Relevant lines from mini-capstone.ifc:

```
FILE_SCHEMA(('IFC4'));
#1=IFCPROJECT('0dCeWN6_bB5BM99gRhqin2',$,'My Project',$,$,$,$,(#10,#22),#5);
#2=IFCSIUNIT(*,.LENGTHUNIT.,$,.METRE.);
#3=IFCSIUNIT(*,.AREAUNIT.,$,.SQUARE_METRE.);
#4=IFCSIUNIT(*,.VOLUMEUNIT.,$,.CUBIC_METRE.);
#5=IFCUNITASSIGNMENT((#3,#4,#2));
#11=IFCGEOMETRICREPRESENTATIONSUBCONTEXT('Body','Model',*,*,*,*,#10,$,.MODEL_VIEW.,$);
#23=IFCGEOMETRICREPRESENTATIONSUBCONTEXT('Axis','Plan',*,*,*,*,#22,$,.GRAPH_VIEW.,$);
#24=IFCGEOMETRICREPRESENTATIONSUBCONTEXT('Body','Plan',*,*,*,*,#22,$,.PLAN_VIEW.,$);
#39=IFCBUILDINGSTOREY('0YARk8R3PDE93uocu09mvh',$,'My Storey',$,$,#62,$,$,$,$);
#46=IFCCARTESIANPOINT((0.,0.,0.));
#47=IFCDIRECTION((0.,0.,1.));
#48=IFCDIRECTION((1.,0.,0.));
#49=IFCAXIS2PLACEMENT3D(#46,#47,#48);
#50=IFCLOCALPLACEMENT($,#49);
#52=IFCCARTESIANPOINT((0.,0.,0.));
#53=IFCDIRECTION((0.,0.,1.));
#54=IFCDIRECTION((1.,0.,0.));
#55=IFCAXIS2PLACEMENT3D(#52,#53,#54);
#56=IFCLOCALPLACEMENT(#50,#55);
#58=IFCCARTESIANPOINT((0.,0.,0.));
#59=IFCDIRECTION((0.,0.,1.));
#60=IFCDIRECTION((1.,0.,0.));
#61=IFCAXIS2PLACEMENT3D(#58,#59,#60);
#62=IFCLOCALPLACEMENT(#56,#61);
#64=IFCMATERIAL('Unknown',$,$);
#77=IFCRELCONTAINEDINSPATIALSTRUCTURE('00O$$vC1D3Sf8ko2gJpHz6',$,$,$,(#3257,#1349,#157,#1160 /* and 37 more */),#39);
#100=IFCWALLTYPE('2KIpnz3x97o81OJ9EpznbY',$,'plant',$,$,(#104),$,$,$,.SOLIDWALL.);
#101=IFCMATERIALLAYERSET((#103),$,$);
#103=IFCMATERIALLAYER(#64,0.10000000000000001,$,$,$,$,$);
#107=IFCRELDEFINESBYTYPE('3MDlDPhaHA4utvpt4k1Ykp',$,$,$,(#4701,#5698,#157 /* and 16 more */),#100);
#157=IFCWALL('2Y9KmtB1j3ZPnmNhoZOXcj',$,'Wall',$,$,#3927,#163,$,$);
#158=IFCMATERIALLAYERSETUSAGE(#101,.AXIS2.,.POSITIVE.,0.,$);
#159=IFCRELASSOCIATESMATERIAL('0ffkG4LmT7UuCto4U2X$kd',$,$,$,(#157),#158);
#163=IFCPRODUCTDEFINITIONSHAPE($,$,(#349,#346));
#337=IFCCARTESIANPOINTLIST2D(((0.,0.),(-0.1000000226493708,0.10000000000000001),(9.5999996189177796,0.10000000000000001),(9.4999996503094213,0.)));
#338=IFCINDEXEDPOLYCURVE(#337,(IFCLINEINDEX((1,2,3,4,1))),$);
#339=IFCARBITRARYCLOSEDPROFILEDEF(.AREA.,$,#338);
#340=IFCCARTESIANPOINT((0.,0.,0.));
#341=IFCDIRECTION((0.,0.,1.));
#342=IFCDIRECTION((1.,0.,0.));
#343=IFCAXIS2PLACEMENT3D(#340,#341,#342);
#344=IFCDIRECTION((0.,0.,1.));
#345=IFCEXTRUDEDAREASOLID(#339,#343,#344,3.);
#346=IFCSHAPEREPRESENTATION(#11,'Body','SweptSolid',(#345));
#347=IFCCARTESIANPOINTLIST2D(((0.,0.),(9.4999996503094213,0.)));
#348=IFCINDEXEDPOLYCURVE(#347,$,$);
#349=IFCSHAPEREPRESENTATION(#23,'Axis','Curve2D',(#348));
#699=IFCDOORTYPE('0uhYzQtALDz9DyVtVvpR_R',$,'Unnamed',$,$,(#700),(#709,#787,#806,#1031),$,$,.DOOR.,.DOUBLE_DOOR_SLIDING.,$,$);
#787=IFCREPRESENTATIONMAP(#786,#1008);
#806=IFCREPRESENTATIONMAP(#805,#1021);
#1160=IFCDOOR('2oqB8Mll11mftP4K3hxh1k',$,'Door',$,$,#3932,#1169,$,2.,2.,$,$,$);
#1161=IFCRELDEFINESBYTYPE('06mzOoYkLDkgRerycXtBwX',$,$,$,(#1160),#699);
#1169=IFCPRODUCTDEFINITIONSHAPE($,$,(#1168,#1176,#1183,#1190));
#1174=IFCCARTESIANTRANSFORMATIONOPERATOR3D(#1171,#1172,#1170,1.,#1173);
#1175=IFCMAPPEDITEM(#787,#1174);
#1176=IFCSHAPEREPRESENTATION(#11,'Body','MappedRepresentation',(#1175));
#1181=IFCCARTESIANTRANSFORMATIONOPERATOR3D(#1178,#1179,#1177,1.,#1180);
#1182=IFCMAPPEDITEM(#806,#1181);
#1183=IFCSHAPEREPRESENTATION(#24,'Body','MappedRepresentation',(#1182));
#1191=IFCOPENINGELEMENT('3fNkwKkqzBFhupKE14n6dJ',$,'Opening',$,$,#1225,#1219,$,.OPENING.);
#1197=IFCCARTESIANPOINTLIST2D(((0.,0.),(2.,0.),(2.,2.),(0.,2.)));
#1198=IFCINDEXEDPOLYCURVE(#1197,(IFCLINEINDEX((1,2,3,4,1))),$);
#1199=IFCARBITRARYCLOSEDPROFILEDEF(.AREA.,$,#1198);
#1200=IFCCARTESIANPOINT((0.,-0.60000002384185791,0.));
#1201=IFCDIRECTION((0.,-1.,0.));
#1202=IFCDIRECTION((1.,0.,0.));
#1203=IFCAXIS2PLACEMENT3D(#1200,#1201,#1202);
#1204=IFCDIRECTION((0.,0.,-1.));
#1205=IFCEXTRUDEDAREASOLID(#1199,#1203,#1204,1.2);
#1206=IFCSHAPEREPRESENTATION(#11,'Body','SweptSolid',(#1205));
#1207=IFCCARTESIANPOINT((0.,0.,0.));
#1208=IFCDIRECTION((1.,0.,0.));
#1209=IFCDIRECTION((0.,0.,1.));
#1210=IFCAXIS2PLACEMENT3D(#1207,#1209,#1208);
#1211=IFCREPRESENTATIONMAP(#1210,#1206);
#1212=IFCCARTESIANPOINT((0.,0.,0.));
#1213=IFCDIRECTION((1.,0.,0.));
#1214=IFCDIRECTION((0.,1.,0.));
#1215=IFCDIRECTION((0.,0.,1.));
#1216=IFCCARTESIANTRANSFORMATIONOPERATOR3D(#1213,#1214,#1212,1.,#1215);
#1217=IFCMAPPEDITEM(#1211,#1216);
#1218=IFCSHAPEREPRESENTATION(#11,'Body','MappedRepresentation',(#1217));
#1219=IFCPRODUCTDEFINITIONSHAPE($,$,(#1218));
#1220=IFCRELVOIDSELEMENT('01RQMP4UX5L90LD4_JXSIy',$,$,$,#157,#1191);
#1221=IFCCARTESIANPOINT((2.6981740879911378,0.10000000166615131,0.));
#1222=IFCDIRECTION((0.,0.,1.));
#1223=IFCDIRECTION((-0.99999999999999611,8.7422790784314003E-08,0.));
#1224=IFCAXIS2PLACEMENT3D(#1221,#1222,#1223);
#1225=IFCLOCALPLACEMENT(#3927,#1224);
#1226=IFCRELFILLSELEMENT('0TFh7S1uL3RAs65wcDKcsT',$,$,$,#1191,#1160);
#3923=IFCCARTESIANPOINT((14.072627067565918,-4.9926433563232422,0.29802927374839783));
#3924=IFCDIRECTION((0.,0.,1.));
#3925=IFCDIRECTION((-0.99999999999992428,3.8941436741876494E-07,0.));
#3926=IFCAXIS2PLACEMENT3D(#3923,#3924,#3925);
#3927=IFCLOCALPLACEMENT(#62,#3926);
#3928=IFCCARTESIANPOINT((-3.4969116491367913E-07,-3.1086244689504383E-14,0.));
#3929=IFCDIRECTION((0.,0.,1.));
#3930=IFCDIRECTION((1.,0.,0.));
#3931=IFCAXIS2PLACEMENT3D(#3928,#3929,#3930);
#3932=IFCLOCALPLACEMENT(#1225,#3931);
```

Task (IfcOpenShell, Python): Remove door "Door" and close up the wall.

```python
import ifcopenshell
import ifcopenshell.api.feature
import ifcopenshell.api.root
import ifcopenshell.geom
import ifcopenshell.util.shape

model = ifcopenshell.open("mini-capstone.ifc")
settings = ifcopenshell.geom.settings()


def volume(element):
    """Net volume in cubic metres, openings subtracted."""
    shape = ifcopenshell.geom.create_shape(settings, element)
    return ifcopenshell.util.shape.get_volume(shape.geometry)


door = model.by_guid("2oqB8Mll11mftP4K3hxh1k")
opening = door.FillsVoids[0].RelatingOpeningElement
wall = opening.VoidsElements[0].RelatingBuildingElement
before = volume(wall)

ifcopenshell.api.root.remove_product(model, product=door)
ifcopenshell.api.feature.remove_feature(model, feature=opening)

after = volume(wall)

print(f"wall volume {before:.3f} -> {after:.3f} m3")

model.write("mini-capstone_rev.ifc")
```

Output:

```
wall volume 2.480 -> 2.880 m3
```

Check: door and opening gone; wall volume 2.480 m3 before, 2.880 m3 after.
